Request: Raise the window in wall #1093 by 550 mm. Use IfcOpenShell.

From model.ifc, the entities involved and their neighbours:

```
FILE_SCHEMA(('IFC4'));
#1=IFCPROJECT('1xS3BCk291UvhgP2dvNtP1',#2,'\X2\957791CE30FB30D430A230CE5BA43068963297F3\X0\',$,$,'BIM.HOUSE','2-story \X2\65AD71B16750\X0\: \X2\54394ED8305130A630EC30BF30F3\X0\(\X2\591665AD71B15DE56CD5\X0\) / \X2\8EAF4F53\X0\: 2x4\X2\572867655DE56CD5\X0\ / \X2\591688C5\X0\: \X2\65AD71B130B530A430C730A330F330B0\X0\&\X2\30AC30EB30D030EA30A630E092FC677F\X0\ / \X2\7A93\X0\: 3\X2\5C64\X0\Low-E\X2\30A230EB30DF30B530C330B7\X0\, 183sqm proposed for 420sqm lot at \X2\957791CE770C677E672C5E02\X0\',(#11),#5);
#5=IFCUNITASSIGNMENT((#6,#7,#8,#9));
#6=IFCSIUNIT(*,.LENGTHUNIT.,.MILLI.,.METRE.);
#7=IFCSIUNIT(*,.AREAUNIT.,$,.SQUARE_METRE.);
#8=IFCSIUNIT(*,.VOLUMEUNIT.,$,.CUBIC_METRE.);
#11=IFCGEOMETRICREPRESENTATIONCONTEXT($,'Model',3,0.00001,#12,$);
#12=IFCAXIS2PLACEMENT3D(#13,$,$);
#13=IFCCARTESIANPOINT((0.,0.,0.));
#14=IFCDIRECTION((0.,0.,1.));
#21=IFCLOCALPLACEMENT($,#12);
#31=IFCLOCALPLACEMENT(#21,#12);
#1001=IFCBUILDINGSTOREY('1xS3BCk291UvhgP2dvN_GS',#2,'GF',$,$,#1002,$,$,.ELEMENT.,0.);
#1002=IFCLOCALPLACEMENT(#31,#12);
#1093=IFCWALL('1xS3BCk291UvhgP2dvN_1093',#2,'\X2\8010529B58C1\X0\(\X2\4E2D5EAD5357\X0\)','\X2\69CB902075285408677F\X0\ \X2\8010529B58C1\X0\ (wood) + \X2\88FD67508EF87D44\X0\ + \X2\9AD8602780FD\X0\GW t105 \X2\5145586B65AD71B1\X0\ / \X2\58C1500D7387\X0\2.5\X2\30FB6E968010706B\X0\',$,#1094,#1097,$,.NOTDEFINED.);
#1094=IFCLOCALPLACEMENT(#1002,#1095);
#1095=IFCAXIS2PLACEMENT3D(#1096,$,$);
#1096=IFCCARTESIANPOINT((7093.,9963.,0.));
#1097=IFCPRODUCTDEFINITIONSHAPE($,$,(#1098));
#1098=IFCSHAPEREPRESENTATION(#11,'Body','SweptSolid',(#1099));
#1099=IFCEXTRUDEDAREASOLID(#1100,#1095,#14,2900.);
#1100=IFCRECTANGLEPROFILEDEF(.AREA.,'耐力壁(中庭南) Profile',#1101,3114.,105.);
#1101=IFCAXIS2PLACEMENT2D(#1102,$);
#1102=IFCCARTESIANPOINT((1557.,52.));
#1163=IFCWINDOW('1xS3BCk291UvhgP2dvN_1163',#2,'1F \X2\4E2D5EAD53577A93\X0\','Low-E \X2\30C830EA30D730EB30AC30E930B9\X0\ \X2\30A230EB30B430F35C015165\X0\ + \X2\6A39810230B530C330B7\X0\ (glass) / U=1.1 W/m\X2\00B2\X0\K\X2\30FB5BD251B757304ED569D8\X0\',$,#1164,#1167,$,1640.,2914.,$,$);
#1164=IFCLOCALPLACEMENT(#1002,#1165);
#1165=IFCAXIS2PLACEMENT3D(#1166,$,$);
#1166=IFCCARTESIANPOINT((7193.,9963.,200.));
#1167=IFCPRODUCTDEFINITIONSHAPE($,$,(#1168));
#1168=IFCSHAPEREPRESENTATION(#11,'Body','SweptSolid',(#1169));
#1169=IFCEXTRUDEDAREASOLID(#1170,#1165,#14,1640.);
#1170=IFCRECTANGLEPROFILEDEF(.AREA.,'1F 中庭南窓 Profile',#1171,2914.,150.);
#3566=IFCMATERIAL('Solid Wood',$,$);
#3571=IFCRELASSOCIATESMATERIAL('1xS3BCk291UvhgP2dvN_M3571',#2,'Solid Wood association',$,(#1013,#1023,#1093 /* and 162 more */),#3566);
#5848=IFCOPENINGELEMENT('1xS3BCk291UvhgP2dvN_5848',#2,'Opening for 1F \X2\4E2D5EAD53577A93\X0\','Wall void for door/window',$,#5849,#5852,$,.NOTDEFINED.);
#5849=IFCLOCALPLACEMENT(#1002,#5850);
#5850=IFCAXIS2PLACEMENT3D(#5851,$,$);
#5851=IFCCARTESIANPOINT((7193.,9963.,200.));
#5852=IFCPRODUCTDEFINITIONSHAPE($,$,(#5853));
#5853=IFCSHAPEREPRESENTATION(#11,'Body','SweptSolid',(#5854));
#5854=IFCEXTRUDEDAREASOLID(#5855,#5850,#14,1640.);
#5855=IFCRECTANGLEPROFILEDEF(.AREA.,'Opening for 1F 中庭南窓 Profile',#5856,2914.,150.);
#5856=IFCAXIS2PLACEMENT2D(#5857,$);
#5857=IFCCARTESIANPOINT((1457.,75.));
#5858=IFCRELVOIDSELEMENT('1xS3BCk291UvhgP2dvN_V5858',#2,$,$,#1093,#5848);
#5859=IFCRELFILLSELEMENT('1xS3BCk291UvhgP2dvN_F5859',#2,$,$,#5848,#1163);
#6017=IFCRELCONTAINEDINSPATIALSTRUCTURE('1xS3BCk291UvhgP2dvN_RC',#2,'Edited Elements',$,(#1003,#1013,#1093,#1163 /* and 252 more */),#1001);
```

```python
import numpy as np
import ifcopenshell
import ifcopenshell.api.geometry
import ifcopenshell.util.placement
import ifcopenshell.util.unit

model = ifcopenshell.open("model.ifc")
unit_scale = ifcopenshell.util.unit.calculate_unit_scale(model)

window = model.by_guid("1xS3BCk291UvhgP2dvN_1163")
opening = window.FillsVoids[0].RelatingOpeningElement
dz = 550.0

shift = np.array([0.0, 0.0, dz])
# The window is not placed relative to its opening, so move both.
for product in (opening, window):
    matrix = ifcopenshell.util.placement.get_local_placement(product.ObjectPlacement)
    matrix[:3, 3] += shift
    ifcopenshell.api.geometry.edit_object_placement(model, product=product, matrix=matrix, is_si=False)

print(f"moved by {dz * unit_scale:+.3f} m")

model.write("model_rev.ifc")
```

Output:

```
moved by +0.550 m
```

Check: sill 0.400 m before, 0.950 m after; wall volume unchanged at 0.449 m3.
